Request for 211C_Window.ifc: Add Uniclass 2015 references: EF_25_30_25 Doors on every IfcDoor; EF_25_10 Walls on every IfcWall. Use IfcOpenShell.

First a look at what the model holds.

```python
import ifcopenshell

model = ifcopenshell.open("211C_Window.ifc")
print(model.schema)
print("classifications:", [c.Name for c in model.by_type("IfcClassification")])
for ifc_class in ("IfcDoor", "IfcRoof", "IfcStair", "IfcWall", "IfcWindow"):
    print(ifc_class, len(model.by_type(ifc_class)))
```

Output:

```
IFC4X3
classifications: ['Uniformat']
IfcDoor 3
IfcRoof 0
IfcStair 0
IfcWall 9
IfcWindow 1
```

```python
import ifcopenshell
import ifcopenshell.api.classification

model = ifcopenshell.open("211C_Window.ifc")

system = ifcopenshell.api.classification.add_classification(model, classification="Uniclass 2015")

codes = {
    "IfcDoor": ("EF_25_30_25", "Doors"),
    "IfcWall": ("EF_25_10", "Walls"),
}
for ifc_class, (code, name) in codes.items():
    products = model.by_type(ifc_class)
    ifcopenshell.api.classification.add_reference(
        model, products=products, classification=system, identification=code, name=name
    )
    print(code, len(products))

model.write("211C_Window_edited.ifc")
```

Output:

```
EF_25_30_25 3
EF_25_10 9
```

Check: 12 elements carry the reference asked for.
